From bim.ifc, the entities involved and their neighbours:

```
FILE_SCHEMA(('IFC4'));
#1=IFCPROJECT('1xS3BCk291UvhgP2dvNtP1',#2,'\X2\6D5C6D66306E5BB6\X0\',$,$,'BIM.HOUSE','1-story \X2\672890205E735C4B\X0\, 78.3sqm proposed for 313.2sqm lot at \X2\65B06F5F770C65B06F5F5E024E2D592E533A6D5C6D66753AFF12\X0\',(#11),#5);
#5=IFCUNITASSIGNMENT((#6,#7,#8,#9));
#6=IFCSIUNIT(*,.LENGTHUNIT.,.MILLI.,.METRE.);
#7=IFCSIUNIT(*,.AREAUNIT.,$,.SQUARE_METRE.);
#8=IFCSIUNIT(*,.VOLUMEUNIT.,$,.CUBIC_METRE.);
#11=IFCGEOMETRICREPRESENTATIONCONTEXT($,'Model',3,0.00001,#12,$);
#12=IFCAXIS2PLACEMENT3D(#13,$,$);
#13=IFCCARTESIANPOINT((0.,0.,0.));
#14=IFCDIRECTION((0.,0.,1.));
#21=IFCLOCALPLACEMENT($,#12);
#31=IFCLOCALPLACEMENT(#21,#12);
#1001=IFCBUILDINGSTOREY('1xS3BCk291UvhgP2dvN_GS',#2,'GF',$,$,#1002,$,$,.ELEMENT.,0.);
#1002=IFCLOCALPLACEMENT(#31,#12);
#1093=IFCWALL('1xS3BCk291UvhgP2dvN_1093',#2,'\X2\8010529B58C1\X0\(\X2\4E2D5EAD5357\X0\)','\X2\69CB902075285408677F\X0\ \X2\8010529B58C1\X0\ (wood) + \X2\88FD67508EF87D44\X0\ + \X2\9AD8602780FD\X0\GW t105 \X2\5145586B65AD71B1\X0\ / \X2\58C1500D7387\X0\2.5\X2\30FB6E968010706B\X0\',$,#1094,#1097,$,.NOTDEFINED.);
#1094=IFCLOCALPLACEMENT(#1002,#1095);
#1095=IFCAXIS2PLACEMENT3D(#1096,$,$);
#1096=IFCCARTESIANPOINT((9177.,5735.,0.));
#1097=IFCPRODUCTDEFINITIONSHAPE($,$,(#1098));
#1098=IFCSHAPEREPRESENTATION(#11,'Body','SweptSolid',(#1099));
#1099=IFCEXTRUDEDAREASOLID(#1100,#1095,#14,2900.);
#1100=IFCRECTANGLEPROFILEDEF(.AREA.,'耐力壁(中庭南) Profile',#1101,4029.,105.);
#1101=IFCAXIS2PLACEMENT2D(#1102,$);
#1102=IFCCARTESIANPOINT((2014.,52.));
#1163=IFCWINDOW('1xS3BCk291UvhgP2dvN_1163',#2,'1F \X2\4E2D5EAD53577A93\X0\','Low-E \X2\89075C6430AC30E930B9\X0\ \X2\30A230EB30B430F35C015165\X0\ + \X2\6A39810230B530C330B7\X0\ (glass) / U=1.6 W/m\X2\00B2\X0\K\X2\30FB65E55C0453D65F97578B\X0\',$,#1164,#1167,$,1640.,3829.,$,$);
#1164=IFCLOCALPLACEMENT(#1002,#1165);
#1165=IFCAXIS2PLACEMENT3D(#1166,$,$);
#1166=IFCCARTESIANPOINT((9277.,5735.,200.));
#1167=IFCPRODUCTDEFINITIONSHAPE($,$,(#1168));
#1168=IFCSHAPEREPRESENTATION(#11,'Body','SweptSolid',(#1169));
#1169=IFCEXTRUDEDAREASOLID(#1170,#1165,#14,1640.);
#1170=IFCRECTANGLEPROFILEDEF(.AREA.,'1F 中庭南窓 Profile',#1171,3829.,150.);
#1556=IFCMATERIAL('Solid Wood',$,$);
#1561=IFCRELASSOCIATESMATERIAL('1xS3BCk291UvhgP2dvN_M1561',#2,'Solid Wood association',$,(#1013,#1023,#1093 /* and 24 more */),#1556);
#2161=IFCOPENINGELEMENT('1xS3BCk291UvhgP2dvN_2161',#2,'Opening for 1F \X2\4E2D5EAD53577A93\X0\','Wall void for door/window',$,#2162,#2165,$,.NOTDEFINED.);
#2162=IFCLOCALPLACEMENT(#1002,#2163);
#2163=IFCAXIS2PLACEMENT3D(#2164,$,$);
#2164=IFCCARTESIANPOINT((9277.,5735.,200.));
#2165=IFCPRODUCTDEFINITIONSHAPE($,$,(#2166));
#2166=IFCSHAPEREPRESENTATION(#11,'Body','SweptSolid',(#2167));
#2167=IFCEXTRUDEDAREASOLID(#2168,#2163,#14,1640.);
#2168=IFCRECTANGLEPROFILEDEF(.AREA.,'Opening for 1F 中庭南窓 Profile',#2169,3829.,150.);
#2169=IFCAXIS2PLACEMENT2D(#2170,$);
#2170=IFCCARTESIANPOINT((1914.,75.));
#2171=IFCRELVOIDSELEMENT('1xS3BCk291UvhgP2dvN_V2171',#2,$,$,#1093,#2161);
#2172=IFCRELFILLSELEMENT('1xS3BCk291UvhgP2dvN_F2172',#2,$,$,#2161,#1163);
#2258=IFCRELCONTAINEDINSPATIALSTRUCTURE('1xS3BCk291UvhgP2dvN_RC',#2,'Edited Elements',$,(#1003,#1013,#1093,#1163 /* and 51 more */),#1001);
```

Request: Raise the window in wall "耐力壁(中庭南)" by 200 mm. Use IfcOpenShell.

```python
import numpy as np
import ifcopenshell
import ifcopenshell.api.geometry
import ifcopenshell.util.placement
import ifcopenshell.util.unit

model = ifcopenshell.open("bim.ifc")
unit_scale = ifcopenshell.util.unit.calculate_unit_scale(model)

window = model.by_guid("1xS3BCk291UvhgP2dvN_1163")
opening = window.FillsVoids[0].RelatingOpeningElement
dz = 0.2 / unit_scale

shift = np.array([0.0, 0.0, dz])
# The window is not placed relative to its opening, so move both.
for product in (opening, window):
    matrix = ifcopenshell.util.placement.get_local_placement(product.ObjectPlacement)
    matrix[:3, 3] += shift
    ifcopenshell.api.geometry.edit_object_placement(model, product=product, matrix=matrix, is_si=False)

print(f"moved by {dz * unit_scale:+.3f} m")

model.write("bim_edited.ifc")
```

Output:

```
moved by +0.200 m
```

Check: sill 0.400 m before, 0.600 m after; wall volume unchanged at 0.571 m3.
